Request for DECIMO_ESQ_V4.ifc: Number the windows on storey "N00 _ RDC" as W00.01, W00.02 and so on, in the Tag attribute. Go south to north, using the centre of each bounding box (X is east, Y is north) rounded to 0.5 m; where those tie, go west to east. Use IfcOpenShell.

First a look at what the model holds.

```python
import ifcopenshell
import ifcopenshell.util.element
import ifcopenshell.util.placement

model = ifcopenshell.open("DECIMO_ESQ_V4.ifc")
print(model.schema)
storey = next(s for s in model.by_type("IfcBuildingStorey") if s.Name == "N00 _ RDC")
windows = [e for e in ifcopenshell.util.element.get_decomposition(storey) if e.is_a("IfcWindow")]
for e in sorted(windows, key=lambda e: e.id()):
    origin = ifcopenshell.util.placement.get_local_placement(e.ObjectPlacement)[:3, 3]
    print(e.id(), e.Tag, e.Name, origin.round(2) + 0.0, sep=" | ")
```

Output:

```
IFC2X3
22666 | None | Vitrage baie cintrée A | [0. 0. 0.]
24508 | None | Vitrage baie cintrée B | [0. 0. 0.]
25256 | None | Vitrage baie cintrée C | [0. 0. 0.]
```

```python
import ifcopenshell
import ifcopenshell.geom
import ifcopenshell.util.element
import ifcopenshell.util.shape

model = ifcopenshell.open("DECIMO_ESQ_V4.ifc")
settings = ifcopenshell.geom.settings()
settings.set("use-world-coords", True)


def centre(element):
    shape = ifcopenshell.geom.create_shape(settings, element)
    return ifcopenshell.util.shape.get_bbox_centroid(shape.geometry)


storey = next(s for s in model.by_type("IfcBuildingStorey") if s.Name == "N00 _ RDC")
windows = [e for e in ifcopenshell.util.element.get_decomposition(storey) if e.is_a("IfcWindow")]

# Insertion points can sit at a corner or the storey origin, so sort by the geometry (in metres).
centres = {e: centre(e) for e in windows}
windows.sort(key=lambda e: (round(centres[e][1] / 0.5), centres[e][0]))

for i, e in enumerate(windows, start=1):
    number = f"W00.{i:02d}"
    e.Tag = number
    print(e.id(), number)

model.write("DECIMO_ESQ_V4_v2.ifc")
```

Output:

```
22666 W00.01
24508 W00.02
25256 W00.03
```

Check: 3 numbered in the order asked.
